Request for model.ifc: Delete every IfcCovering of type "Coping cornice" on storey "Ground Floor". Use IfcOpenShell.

First a look at what the model holds.

```python
import ifcopenshell
import ifcopenshell.util.element

model = ifcopenshell.open("model.ifc")
print(model.schema)
storey = next(s for s in model.by_type("IfcBuildingStorey") if s.Name == "Ground Floor")
coverings = [e for e in ifcopenshell.util.element.get_decomposition(storey) if e.is_a("IfcCovering")]
seen = {}
for e in coverings:
    element_type = ifcopenshell.util.element.get_type(e)
    name = element_type.Name if element_type not in (None, e) else None
    seen[name] = seen.get(name, 0) + 1
for name, count in sorted(seen.items(), key=str):
    print(count, "x", name)
```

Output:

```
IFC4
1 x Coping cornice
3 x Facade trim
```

```python
import ifcopenshell
import ifcopenshell.api.root
import ifcopenshell.util.element

model = ifcopenshell.open("model.ifc")

storey = next(s for s in model.by_type("IfcBuildingStorey") if s.Name == "Ground Floor")
coverings = [e for e in ifcopenshell.util.element.get_decomposition(storey) if e.is_a("IfcCovering")]
targets = [e for e in coverings if (t := ifcopenshell.util.element.get_type(e)) not in (None, e) and t.Name == "Coping cornice"]

for e in targets:
    ifcopenshell.api.root.remove_product(model, product=e)
print(len(targets), "removed")

model.write("model_v2.ifc")
```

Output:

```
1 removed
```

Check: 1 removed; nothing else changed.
